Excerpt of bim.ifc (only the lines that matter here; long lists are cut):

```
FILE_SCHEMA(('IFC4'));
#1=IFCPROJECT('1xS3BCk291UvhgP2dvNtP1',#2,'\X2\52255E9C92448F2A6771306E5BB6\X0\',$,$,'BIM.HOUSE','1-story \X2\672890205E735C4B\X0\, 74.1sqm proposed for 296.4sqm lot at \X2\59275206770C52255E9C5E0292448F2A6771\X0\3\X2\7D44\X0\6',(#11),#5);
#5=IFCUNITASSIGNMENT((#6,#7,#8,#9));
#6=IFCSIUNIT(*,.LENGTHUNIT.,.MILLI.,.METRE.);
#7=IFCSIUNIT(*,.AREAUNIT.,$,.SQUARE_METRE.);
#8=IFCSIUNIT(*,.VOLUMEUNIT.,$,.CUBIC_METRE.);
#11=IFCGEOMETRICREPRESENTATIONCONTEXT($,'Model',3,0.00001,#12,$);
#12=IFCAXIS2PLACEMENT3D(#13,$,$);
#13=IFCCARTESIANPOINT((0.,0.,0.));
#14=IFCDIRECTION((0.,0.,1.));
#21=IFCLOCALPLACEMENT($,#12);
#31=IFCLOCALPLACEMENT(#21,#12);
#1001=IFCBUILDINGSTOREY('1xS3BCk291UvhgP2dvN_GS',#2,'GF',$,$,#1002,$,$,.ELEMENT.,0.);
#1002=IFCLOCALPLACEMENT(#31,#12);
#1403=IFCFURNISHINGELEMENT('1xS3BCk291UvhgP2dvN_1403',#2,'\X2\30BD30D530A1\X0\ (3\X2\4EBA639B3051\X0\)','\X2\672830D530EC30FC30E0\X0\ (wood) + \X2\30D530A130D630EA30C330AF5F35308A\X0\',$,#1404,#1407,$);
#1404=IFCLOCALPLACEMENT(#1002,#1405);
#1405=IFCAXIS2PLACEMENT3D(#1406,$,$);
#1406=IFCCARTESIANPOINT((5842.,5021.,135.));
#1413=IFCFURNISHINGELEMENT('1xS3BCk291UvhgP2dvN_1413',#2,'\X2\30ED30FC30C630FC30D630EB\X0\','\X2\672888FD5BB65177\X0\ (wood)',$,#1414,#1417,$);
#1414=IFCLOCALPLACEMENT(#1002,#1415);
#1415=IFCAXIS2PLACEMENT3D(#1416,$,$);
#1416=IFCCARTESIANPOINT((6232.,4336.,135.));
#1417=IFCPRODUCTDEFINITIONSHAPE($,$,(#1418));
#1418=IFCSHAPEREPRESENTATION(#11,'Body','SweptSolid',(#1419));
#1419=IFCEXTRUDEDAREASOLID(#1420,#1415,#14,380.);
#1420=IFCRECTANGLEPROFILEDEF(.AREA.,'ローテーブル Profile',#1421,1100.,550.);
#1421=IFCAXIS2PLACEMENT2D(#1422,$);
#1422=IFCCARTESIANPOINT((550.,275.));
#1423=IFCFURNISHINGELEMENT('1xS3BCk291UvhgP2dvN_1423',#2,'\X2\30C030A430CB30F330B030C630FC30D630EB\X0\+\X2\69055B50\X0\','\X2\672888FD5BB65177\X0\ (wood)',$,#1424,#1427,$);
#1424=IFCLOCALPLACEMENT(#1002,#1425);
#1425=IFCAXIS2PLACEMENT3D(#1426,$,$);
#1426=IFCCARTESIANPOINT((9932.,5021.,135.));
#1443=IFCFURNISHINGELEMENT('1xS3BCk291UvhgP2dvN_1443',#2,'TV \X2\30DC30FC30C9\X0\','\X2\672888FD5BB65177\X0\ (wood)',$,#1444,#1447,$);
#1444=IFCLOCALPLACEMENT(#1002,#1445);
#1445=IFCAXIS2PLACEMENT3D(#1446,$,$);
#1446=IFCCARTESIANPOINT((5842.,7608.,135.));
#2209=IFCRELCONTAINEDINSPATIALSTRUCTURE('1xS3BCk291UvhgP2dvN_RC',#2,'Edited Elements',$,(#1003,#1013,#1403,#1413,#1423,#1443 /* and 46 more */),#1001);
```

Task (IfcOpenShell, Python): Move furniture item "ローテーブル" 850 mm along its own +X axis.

```python
import ifcopenshell
import ifcopenshell.api.geometry
import ifcopenshell.util.placement
import ifcopenshell.util.unit

model = ifcopenshell.open("bim.ifc")
unit_scale = ifcopenshell.util.unit.calculate_unit_scale(model)

item = model.by_guid("1xS3BCk291UvhgP2dvN_1413")
matrix = ifcopenshell.util.placement.get_local_placement(item.ObjectPlacement)
matrix[:3, 3] += matrix[:3, 0] * 0.85 / unit_scale
ifcopenshell.api.geometry.edit_object_placement(model, product=item, matrix=matrix, is_si=False)

print(ifcopenshell.util.placement.get_local_placement(item.ObjectPlacement).round(3) + 0.0)

model.write("bim_rev.ifc")
```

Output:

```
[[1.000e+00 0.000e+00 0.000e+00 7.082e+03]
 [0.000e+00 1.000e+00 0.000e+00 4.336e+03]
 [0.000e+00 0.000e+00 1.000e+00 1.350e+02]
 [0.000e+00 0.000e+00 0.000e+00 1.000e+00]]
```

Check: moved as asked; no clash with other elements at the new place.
